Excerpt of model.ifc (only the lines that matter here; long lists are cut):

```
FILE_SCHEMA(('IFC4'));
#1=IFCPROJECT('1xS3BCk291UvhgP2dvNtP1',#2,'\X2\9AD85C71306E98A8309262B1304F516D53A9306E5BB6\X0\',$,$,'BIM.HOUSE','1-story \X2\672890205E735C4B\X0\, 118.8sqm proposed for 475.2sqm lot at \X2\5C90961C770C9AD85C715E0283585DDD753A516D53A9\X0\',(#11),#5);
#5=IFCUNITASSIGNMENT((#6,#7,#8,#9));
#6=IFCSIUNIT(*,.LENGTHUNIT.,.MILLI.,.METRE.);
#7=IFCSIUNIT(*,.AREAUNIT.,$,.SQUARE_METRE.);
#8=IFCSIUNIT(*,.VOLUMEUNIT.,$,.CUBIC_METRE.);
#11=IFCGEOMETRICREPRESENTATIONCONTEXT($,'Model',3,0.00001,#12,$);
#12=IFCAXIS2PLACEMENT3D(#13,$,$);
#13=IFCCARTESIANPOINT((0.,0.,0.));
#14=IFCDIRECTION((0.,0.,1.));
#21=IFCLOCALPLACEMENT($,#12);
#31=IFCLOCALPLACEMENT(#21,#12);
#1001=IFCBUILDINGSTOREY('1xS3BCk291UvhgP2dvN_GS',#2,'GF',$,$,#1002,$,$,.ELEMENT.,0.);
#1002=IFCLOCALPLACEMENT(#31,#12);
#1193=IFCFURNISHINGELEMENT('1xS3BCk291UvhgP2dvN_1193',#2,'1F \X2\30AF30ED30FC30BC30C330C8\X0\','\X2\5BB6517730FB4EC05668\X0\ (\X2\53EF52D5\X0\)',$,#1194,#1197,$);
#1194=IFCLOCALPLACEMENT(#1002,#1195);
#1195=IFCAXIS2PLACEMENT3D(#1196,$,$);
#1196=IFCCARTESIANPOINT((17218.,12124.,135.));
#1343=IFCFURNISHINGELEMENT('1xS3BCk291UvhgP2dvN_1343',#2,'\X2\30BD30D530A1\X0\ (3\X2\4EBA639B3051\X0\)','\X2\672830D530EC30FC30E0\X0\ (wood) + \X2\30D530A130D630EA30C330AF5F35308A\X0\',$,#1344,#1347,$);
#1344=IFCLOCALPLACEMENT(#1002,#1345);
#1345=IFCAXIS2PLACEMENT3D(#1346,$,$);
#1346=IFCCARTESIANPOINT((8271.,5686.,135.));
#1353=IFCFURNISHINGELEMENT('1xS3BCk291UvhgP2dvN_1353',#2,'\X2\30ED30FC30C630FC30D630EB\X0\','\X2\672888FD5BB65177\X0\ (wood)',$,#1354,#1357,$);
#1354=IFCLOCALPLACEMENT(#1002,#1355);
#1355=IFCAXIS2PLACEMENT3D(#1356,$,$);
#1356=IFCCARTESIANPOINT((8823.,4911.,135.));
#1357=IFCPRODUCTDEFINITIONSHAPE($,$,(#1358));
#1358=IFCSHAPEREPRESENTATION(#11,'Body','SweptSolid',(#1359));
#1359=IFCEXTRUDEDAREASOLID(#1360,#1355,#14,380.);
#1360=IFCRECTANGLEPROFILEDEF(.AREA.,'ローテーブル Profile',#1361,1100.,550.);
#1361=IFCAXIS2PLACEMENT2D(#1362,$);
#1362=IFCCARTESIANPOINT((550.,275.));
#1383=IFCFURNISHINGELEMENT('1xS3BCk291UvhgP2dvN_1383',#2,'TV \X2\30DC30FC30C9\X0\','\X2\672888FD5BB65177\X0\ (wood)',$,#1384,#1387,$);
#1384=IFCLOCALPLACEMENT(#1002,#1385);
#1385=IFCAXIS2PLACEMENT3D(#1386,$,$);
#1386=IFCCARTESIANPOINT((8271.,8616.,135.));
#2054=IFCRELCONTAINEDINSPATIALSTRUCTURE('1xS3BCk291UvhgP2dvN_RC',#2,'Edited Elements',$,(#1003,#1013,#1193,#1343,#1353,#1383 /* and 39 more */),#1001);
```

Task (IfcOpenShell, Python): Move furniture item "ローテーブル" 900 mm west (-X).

```python
import ifcopenshell
import ifcopenshell.api.geometry
import ifcopenshell.util.placement

model = ifcopenshell.open("model.ifc")

item = model.by_id(1353)
matrix = ifcopenshell.util.placement.get_local_placement(item.ObjectPlacement)
matrix[0, 3] -= 900.0
ifcopenshell.api.geometry.edit_object_placement(model, product=item, matrix=matrix, is_si=False)

print(ifcopenshell.util.placement.get_local_placement(item.ObjectPlacement).round(3) + 0.0)

model.write("model_edited.ifc")
```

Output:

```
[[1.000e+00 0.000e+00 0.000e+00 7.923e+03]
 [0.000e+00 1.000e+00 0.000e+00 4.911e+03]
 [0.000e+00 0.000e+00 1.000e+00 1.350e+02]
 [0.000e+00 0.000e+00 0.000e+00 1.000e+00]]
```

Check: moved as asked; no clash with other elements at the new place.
